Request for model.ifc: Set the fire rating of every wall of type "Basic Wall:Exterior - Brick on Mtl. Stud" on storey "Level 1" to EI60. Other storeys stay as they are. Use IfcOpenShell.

First a look at what the model holds.

```python
import ifcopenshell
import ifcopenshell.util.element

model = ifcopenshell.open("model.ifc")
print(model.schema)
storey = next(s for s in model.by_type("IfcBuildingStorey") if s.Name == "Level 1")
walls = [e for e in ifcopenshell.util.element.get_decomposition(storey) if e.is_a("IfcWall")]
seen = {}
for e in walls:
    element_type = ifcopenshell.util.element.get_type(e)
    key = (element_type.Name if element_type != e and element_type else None, ifcopenshell.util.element.get_pset(e, "Pset_WallCommon", "FireRating"))
    seen[key] = seen.get(key, 0) + 1
for (name, value), count in sorted(seen.items(), key=str):
    print(count, "x", name, "|", value)
```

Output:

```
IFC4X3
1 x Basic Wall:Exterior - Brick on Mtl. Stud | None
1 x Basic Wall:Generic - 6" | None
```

```python
import ifcopenshell
import ifcopenshell.api.pset
import ifcopenshell.util.element

model = ifcopenshell.open("model.ifc")

storey = next(s for s in model.by_type("IfcBuildingStorey") if s.Name == "Level 1")
walls = [e for e in ifcopenshell.util.element.get_decomposition(storey) if e.is_a("IfcWall")]

count = 0
for e in walls:
    element_type = ifcopenshell.util.element.get_type(e)
    if element_type in (None, e) or element_type.Name != "Basic Wall:Exterior - Brick on Mtl. Stud":
        continue
    # add_pset returns the element's existing set when there is one.
    pset = ifcopenshell.api.pset.add_pset(model, product=e, name="Pset_WallCommon")
    ifcopenshell.api.pset.edit_pset(model, pset=pset, properties={"FireRating": "EI60"})
    count += 1

print(count, "walls updated")

model.write("model_v2.ifc")
```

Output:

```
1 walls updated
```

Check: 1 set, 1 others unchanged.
